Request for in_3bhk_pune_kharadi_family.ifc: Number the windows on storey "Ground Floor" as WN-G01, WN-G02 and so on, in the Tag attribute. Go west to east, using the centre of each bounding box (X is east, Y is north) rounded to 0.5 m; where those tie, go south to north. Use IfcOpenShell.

First a look at what the model holds.

```python
import ifcopenshell
import ifcopenshell.util.element
import ifcopenshell.util.placement

model = ifcopenshell.open("in_3bhk_pune_kharadi_family.ifc")
print(model.schema)
storey = next(s for s in model.by_type("IfcBuildingStorey") if s.Name == "Ground Floor")
windows = [e for e in ifcopenshell.util.element.get_decomposition(storey) if e.is_a("IfcWindow")]
for e in sorted(windows, key=lambda e: e.id()):
    origin = ifcopenshell.util.placement.get_local_placement(e.ObjectPlacement)[:3, 3]
    print(e.id(), e.Tag, e.Name, origin.round(2) + 0.0, sep=" | ")
```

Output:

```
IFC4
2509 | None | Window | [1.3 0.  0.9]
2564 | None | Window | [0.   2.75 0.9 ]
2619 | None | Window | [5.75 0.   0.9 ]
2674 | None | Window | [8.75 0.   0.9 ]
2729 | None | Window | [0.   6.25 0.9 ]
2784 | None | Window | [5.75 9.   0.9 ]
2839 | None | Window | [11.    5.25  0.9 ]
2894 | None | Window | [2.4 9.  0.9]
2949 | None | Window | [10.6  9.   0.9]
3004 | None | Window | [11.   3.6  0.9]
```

```python
import ifcopenshell
import ifcopenshell.geom
import ifcopenshell.util.element
import ifcopenshell.util.shape

model = ifcopenshell.open("in_3bhk_pune_kharadi_family.ifc")
settings = ifcopenshell.geom.settings()
settings.set("use-world-coords", True)


def centre(element):
    shape = ifcopenshell.geom.create_shape(settings, element)
    return ifcopenshell.util.shape.get_bbox_centroid(shape.geometry)


storey = next(s for s in model.by_type("IfcBuildingStorey") if s.Name == "Ground Floor")
windows = [e for e in ifcopenshell.util.element.get_decomposition(storey) if e.is_a("IfcWindow")]

# Insertion points can sit at a corner or the storey origin, so sort by the geometry (in metres).
centres = {e: centre(e) for e in windows}
windows.sort(key=lambda e: (round(centres[e][0] / 0.5), centres[e][1]))

for i, e in enumerate(windows, start=1):
    number = f"WN-G{i:02d}"
    e.Tag = number
    print(e.id(), number)

model.write("in_3bhk_pune_kharadi_family_v2.ifc")
```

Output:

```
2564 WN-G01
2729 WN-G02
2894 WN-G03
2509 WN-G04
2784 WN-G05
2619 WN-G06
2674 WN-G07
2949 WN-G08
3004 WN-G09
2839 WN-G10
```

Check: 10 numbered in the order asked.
